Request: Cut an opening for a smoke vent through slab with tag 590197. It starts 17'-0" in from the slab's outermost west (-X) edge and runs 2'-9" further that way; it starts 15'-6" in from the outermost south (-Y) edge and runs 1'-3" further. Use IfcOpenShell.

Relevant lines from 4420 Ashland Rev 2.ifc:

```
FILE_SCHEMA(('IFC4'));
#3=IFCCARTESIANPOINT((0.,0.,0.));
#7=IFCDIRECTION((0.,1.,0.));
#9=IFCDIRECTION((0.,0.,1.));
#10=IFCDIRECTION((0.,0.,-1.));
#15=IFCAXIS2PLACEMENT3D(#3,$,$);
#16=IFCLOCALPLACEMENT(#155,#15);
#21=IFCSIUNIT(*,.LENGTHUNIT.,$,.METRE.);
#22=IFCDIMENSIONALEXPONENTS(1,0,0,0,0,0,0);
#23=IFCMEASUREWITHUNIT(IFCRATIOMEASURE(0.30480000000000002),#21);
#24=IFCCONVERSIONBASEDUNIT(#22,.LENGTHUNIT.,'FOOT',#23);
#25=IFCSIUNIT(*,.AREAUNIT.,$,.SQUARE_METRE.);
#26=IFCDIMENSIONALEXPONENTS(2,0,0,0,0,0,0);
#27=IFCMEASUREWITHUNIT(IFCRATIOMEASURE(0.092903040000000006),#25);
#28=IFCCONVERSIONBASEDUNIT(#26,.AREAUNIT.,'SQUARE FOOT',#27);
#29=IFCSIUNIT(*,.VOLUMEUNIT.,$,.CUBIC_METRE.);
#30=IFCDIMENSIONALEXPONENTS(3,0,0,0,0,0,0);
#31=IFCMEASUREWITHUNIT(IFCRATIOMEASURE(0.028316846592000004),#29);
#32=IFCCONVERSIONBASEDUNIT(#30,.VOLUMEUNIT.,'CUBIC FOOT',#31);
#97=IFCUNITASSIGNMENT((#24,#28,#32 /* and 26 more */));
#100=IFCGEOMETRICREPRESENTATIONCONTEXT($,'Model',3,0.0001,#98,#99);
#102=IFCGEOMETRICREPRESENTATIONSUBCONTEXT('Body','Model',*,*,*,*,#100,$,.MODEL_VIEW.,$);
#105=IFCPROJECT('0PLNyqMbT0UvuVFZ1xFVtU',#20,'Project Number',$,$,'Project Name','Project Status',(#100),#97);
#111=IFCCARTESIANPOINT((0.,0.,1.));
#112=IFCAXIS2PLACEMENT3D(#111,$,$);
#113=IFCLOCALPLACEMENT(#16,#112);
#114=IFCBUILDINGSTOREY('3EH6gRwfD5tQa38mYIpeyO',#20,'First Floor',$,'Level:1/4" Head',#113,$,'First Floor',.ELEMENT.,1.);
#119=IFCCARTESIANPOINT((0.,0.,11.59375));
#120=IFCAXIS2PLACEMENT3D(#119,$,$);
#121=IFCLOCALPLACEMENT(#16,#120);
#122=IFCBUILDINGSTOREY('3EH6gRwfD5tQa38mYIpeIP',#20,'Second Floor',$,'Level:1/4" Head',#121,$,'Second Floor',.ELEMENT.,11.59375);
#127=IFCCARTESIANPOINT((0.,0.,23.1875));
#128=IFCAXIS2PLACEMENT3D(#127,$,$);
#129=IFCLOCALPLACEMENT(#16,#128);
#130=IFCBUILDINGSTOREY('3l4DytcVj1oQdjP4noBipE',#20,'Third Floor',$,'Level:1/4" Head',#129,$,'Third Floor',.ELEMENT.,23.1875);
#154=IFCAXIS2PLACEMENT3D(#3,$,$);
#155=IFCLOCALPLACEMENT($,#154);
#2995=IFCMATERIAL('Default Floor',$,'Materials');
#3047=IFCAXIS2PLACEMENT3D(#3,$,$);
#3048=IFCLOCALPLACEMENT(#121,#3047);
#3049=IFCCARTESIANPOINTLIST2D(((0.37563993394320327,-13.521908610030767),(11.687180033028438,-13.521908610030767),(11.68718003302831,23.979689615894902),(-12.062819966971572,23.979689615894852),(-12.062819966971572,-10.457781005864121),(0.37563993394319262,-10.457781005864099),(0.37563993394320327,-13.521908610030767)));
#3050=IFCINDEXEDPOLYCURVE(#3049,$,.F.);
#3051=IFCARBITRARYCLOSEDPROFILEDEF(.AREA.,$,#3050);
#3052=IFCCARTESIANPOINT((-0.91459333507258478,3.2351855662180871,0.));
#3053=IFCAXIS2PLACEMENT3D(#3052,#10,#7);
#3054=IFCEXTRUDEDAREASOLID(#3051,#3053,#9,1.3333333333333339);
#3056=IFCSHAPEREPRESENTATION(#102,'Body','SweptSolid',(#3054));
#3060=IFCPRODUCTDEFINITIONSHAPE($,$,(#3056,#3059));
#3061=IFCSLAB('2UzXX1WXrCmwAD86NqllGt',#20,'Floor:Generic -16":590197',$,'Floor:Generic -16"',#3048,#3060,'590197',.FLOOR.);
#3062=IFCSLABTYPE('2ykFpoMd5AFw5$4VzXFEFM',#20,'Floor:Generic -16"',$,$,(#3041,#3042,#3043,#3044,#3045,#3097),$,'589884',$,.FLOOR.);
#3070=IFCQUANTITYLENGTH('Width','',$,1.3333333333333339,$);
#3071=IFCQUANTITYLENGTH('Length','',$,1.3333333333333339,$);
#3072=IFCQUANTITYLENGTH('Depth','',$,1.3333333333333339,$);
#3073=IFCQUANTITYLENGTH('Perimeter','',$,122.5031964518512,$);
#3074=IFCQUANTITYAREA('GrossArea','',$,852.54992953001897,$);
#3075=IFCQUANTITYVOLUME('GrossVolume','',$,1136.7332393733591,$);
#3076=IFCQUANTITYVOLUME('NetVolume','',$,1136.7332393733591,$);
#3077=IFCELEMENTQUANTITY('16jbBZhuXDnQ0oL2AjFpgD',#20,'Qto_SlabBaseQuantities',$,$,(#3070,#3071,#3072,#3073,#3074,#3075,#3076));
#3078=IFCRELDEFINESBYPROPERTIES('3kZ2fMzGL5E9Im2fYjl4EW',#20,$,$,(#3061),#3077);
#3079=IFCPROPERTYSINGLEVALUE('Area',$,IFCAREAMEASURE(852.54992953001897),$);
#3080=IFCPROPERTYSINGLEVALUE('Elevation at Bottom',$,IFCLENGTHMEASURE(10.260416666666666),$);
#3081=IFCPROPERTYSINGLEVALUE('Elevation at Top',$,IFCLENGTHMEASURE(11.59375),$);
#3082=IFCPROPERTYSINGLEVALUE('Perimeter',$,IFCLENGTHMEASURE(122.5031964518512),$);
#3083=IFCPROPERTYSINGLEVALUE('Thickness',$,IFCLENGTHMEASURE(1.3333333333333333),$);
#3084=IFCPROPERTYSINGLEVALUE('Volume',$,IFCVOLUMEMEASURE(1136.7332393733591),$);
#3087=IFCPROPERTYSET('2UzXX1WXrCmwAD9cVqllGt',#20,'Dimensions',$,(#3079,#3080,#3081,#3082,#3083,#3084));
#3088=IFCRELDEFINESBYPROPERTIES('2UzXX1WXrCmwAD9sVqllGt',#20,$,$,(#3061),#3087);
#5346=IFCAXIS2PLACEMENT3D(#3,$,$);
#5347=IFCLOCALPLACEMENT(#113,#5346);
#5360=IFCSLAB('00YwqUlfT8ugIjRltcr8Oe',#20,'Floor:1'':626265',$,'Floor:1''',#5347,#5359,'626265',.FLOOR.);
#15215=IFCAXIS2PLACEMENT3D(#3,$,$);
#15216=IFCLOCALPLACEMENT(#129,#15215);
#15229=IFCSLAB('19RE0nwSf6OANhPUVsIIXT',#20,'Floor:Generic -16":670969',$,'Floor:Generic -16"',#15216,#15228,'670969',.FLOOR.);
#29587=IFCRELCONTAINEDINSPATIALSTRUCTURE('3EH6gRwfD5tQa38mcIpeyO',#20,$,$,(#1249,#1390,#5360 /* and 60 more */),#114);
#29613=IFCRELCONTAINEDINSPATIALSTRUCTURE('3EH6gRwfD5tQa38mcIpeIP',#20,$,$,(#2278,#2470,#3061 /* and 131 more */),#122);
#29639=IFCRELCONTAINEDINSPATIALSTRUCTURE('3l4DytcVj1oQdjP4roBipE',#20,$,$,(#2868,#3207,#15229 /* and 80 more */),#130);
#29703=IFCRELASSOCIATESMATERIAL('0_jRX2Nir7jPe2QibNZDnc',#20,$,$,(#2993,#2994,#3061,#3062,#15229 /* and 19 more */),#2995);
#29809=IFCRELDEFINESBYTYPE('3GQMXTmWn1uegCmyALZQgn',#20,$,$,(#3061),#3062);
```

```python
import numpy as np
import ifcopenshell
import ifcopenshell.api.feature
import ifcopenshell.api.geometry
import ifcopenshell.api.pset
import ifcopenshell.api.root
import ifcopenshell.geom
import ifcopenshell.util.element
import ifcopenshell.util.placement
import ifcopenshell.util.representation
import ifcopenshell.util.shape
import ifcopenshell.util.unit

model = ifcopenshell.open("4420 Ashland Rev 2.ifc")
unit_scale = ifcopenshell.util.unit.calculate_unit_scale(model)
area_scale = ifcopenshell.util.unit.calculate_unit_scale(model, "AREAUNIT")
volume_scale = ifcopenshell.util.unit.calculate_unit_scale(model, "VOLUMEUNIT")
settings = ifcopenshell.geom.settings()


def volume(element):
    """Net volume in cubic metres, openings subtracted."""
    shape = ifcopenshell.geom.create_shape(settings, element)
    return ifcopenshell.util.shape.get_volume(shape.geometry)


slab = model.by_guid("2UzXX1WXrCmwAD86NqllGt")
before = volume(slab)

# Extent in the slab's own axes, in metres. The edges named are its -X and -Y sides.
slab_shape = ifcopenshell.geom.create_shape(settings, slab)
vertices = ifcopenshell.util.shape.get_vertices(slab_shape.geometry)
x_min, y_min, bottom = vertices.min(axis=0)
top = vertices[:, 2].max()

opening = ifcopenshell.api.root.create_entity(model, ifc_class="IfcOpeningElement", name="Smoke vent opening", predefined_type="OPENING")
context = ifcopenshell.util.representation.get_context(model, "Model", "Body", "MODEL_VIEW")
width, depth = 0.8382, 0.381
outline = [(0.0, 0.0), (width, 0.0), (width, depth), (0.0, depth), (0.0, 0.0)]
# Overshoot both faces by 50 mm so the cut is clean.
shape = ifcopenshell.api.geometry.add_slab_representation(
    model, context=context, depth=top - bottom + 0.1, polyline=outline
)
ifcopenshell.api.geometry.assign_representation(model, product=opening, representation=shape)

matrix = ifcopenshell.util.placement.get_local_placement(slab.ObjectPlacement)
matrix[:, 3] = matrix @ np.append(np.array([x_min + 5.1816, y_min + 4.7244, bottom - 0.05]) / unit_scale, 1.0)
ifcopenshell.api.geometry.edit_object_placement(model, product=opening, matrix=matrix, is_si=False)
ifcopenshell.api.feature.add_feature(model, feature=opening, element=slab)

after = volume(slab)

# Update the slab's stored quantities.
qto = model.by_id(ifcopenshell.util.element.get_pset(slab, "Qto_SlabBaseQuantities", should_inherit=False)["id"])
ifcopenshell.api.pset.edit_qto(model, qto=qto, properties={"NetVolume": after / volume_scale})
pset = model.by_id(ifcopenshell.util.element.get_pset(slab, "Dimensions", should_inherit=False)["id"])
ifcopenshell.api.pset.edit_pset(model, pset=pset, properties={
    "Area": model.create_entity("IfcAreaMeasure", after / (top - bottom) / area_scale),
    "Volume": model.create_entity("IfcVolumeMeasure", after / volume_scale),
})

print(f"slab volume {before:.3f} -> {after:.3f} m3")

model.write("4420 Ashland Rev 2_v2.ifc")
```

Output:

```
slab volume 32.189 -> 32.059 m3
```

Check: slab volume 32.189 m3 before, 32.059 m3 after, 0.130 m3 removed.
